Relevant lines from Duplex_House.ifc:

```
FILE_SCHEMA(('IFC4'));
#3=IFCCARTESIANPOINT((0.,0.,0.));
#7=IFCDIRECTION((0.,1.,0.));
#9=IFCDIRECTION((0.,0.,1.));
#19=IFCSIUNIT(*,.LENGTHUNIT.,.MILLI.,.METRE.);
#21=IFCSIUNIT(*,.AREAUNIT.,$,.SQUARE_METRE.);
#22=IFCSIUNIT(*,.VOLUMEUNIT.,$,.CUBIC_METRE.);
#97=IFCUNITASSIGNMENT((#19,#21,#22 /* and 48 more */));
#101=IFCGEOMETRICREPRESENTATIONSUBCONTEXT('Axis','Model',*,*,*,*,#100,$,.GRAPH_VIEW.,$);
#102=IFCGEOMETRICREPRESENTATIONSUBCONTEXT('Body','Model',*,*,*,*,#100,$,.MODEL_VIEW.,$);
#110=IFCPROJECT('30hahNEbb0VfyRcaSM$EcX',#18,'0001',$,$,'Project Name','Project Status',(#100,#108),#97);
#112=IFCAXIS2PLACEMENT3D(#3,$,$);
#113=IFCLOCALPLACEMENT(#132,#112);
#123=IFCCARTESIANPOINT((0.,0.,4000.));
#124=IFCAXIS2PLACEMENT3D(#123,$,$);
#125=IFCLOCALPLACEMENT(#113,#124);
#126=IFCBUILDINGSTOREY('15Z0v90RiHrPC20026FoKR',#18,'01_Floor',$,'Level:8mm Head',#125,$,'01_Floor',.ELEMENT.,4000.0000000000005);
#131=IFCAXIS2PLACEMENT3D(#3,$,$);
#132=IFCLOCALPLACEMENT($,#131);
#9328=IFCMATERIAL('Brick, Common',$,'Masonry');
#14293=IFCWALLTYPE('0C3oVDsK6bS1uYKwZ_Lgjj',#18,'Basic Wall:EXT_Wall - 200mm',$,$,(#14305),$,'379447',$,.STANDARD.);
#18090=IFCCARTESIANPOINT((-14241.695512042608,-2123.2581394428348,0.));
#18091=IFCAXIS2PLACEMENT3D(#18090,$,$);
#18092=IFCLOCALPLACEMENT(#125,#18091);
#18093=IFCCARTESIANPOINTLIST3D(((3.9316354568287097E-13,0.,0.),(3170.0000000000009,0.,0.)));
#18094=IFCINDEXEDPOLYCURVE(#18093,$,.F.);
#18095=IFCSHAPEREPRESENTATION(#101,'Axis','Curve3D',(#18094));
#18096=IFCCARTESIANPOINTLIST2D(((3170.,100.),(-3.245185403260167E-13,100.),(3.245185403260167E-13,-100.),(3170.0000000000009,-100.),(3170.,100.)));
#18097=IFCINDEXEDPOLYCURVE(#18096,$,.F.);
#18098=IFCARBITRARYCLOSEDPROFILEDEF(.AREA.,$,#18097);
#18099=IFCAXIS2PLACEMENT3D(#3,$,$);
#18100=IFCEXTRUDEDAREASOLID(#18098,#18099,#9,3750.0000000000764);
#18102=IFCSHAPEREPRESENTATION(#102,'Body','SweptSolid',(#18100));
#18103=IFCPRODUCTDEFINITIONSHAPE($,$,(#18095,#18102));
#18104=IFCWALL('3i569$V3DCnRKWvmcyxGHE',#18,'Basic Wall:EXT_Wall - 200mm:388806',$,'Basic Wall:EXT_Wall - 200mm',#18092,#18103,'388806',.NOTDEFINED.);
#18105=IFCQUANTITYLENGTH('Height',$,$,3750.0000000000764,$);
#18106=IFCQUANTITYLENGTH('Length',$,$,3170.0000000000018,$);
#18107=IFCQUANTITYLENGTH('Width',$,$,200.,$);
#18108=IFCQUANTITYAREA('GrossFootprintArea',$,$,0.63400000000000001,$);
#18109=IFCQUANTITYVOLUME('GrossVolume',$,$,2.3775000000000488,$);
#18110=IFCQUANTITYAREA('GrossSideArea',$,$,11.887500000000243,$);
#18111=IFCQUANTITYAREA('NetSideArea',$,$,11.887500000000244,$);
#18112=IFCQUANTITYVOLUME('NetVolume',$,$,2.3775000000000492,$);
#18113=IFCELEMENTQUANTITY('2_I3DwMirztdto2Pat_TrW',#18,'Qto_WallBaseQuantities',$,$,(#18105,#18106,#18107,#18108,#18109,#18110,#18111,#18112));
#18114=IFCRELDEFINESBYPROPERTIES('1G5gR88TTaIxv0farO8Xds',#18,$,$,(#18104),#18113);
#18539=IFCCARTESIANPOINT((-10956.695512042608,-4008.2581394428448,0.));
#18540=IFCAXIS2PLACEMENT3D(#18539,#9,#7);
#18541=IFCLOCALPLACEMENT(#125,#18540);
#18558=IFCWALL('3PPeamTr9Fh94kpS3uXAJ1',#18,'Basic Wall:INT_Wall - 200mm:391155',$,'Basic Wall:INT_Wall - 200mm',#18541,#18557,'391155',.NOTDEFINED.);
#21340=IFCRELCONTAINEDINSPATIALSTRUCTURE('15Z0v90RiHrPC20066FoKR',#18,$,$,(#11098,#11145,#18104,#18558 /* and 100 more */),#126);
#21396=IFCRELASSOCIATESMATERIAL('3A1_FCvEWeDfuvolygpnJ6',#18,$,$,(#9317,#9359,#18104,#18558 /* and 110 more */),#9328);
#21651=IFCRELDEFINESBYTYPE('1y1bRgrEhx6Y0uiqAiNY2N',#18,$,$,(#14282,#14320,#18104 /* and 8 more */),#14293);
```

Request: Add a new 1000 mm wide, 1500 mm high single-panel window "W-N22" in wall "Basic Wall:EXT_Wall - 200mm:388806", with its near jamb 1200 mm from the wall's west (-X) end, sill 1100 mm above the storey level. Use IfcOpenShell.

```python
import numpy as np
import ifcopenshell
import ifcopenshell.api.feature
import ifcopenshell.api.geometry
import ifcopenshell.api.pset
import ifcopenshell.api.root
import ifcopenshell.api.spatial
import ifcopenshell.geom
import ifcopenshell.util.element
import ifcopenshell.util.placement
import ifcopenshell.util.representation
import ifcopenshell.util.shape
import ifcopenshell.util.unit

model = ifcopenshell.open("Duplex_House.ifc")
unit_scale = ifcopenshell.util.unit.calculate_unit_scale(model)
area_scale = ifcopenshell.util.unit.calculate_unit_scale(model, "AREAUNIT")
volume_scale = ifcopenshell.util.unit.calculate_unit_scale(model, "VOLUMEUNIT")
settings = ifcopenshell.geom.settings()


def volume(element):
    """Net volume in cubic metres, openings subtracted."""
    shape = ifcopenshell.geom.create_shape(settings, element)
    return ifcopenshell.util.shape.get_volume(shape.geometry)


wall = model.by_guid("3i569$V3DCnRKWvmcyxGHE")
storey = ifcopenshell.util.element.get_container(wall, ifc_class="IfcBuildingStorey")
context = ifcopenshell.util.representation.get_context(model, "Model", "Body", "MODEL_VIEW")
before = volume(wall)

width, height, from_end, sill = 1, 1.5, 1.2, 1.1  # metres

# The wall runs along its own X axis, and the end named is its -X end.
wall_shape = ifcopenshell.geom.create_shape(settings, wall)
x, y, z = ifcopenshell.util.shape.get_vertices(wall_shape.geometry).T
start = x.min() + from_end
face, thickness = float(y.min()), float(y.max() - y.min())
wall_matrix = ifcopenshell.util.placement.get_local_placement(wall.ObjectPlacement)
level = ifcopenshell.util.placement.get_local_placement(storey.ObjectPlacement)[2, 3]


def in_wall(x, y):
    """Placement at x, y metres in the wall's axes, at sill height."""
    matrix = wall_matrix.copy()
    matrix[:, 3] = wall_matrix @ np.array([x / unit_scale, y / unit_scale, 0.0, 1.0])
    matrix[2, 3] = level + sill / unit_scale
    return matrix


# Opening: a box that overshoots both wall faces by 50 mm.
opening = ifcopenshell.api.root.create_entity(model, ifc_class="IfcOpeningElement", predefined_type="OPENING")
box = ifcopenshell.api.geometry.add_wall_representation(
    model, context=context, length=width, height=height, thickness=thickness + 0.1
)
ifcopenshell.api.geometry.assign_representation(model, product=opening, representation=box)
ifcopenshell.api.geometry.edit_object_placement(model, product=opening, matrix=in_wall(start, face - 0.05), is_si=False)
ifcopenshell.api.feature.add_feature(model, feature=opening, element=wall)

window = ifcopenshell.api.root.create_entity(model, ifc_class="IfcWindow", name="W-N22", predefined_type="WINDOW")
window.OverallWidth, window.OverallHeight = width / unit_scale, height / unit_scale
window.PartitioningType = "SINGLE_PANEL"
body = ifcopenshell.api.geometry.add_window_representation(
    model,
    context=context,
    overall_width=window.OverallWidth,
    overall_height=window.OverallHeight,
    partition_type="SINGLE_PANEL",
)
ifcopenshell.api.geometry.assign_representation(model, product=window, representation=body)
ifcopenshell.api.spatial.assign_container(model, products=[window], relating_structure=storey)
ifcopenshell.api.feature.add_filling(model, opening=opening, element=window)

# Centre the window in the wall's thickness.
ifcopenshell.api.geometry.edit_object_placement(model, product=window, matrix=in_wall(start, face), is_si=False)
window_shape = ifcopenshell.geom.create_shape(settings, window)
depth = ifcopenshell.util.shape.get_vertices(window_shape.geometry)[:, 1]
offset = face + thickness / 2 - (depth.min() + depth.max()) / 2
ifcopenshell.api.geometry.edit_object_placement(model, product=window, matrix=in_wall(start, offset), is_si=False)

after = volume(wall)

# Update the wall's stored quantities.
qto = model.by_id(ifcopenshell.util.element.get_pset(wall, "Qto_WallBaseQuantities", should_inherit=False)["id"])
ifcopenshell.api.pset.edit_qto(model, qto=qto, properties={
    "NetSideArea": after / thickness / area_scale,
    "NetVolume": after / volume_scale,
})

print(f"wall volume {before:.3f} -> {after:.3f} m3")

model.write("Duplex_House_edited.ifc")
```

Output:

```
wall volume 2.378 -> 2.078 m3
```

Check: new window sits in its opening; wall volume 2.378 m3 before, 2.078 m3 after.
